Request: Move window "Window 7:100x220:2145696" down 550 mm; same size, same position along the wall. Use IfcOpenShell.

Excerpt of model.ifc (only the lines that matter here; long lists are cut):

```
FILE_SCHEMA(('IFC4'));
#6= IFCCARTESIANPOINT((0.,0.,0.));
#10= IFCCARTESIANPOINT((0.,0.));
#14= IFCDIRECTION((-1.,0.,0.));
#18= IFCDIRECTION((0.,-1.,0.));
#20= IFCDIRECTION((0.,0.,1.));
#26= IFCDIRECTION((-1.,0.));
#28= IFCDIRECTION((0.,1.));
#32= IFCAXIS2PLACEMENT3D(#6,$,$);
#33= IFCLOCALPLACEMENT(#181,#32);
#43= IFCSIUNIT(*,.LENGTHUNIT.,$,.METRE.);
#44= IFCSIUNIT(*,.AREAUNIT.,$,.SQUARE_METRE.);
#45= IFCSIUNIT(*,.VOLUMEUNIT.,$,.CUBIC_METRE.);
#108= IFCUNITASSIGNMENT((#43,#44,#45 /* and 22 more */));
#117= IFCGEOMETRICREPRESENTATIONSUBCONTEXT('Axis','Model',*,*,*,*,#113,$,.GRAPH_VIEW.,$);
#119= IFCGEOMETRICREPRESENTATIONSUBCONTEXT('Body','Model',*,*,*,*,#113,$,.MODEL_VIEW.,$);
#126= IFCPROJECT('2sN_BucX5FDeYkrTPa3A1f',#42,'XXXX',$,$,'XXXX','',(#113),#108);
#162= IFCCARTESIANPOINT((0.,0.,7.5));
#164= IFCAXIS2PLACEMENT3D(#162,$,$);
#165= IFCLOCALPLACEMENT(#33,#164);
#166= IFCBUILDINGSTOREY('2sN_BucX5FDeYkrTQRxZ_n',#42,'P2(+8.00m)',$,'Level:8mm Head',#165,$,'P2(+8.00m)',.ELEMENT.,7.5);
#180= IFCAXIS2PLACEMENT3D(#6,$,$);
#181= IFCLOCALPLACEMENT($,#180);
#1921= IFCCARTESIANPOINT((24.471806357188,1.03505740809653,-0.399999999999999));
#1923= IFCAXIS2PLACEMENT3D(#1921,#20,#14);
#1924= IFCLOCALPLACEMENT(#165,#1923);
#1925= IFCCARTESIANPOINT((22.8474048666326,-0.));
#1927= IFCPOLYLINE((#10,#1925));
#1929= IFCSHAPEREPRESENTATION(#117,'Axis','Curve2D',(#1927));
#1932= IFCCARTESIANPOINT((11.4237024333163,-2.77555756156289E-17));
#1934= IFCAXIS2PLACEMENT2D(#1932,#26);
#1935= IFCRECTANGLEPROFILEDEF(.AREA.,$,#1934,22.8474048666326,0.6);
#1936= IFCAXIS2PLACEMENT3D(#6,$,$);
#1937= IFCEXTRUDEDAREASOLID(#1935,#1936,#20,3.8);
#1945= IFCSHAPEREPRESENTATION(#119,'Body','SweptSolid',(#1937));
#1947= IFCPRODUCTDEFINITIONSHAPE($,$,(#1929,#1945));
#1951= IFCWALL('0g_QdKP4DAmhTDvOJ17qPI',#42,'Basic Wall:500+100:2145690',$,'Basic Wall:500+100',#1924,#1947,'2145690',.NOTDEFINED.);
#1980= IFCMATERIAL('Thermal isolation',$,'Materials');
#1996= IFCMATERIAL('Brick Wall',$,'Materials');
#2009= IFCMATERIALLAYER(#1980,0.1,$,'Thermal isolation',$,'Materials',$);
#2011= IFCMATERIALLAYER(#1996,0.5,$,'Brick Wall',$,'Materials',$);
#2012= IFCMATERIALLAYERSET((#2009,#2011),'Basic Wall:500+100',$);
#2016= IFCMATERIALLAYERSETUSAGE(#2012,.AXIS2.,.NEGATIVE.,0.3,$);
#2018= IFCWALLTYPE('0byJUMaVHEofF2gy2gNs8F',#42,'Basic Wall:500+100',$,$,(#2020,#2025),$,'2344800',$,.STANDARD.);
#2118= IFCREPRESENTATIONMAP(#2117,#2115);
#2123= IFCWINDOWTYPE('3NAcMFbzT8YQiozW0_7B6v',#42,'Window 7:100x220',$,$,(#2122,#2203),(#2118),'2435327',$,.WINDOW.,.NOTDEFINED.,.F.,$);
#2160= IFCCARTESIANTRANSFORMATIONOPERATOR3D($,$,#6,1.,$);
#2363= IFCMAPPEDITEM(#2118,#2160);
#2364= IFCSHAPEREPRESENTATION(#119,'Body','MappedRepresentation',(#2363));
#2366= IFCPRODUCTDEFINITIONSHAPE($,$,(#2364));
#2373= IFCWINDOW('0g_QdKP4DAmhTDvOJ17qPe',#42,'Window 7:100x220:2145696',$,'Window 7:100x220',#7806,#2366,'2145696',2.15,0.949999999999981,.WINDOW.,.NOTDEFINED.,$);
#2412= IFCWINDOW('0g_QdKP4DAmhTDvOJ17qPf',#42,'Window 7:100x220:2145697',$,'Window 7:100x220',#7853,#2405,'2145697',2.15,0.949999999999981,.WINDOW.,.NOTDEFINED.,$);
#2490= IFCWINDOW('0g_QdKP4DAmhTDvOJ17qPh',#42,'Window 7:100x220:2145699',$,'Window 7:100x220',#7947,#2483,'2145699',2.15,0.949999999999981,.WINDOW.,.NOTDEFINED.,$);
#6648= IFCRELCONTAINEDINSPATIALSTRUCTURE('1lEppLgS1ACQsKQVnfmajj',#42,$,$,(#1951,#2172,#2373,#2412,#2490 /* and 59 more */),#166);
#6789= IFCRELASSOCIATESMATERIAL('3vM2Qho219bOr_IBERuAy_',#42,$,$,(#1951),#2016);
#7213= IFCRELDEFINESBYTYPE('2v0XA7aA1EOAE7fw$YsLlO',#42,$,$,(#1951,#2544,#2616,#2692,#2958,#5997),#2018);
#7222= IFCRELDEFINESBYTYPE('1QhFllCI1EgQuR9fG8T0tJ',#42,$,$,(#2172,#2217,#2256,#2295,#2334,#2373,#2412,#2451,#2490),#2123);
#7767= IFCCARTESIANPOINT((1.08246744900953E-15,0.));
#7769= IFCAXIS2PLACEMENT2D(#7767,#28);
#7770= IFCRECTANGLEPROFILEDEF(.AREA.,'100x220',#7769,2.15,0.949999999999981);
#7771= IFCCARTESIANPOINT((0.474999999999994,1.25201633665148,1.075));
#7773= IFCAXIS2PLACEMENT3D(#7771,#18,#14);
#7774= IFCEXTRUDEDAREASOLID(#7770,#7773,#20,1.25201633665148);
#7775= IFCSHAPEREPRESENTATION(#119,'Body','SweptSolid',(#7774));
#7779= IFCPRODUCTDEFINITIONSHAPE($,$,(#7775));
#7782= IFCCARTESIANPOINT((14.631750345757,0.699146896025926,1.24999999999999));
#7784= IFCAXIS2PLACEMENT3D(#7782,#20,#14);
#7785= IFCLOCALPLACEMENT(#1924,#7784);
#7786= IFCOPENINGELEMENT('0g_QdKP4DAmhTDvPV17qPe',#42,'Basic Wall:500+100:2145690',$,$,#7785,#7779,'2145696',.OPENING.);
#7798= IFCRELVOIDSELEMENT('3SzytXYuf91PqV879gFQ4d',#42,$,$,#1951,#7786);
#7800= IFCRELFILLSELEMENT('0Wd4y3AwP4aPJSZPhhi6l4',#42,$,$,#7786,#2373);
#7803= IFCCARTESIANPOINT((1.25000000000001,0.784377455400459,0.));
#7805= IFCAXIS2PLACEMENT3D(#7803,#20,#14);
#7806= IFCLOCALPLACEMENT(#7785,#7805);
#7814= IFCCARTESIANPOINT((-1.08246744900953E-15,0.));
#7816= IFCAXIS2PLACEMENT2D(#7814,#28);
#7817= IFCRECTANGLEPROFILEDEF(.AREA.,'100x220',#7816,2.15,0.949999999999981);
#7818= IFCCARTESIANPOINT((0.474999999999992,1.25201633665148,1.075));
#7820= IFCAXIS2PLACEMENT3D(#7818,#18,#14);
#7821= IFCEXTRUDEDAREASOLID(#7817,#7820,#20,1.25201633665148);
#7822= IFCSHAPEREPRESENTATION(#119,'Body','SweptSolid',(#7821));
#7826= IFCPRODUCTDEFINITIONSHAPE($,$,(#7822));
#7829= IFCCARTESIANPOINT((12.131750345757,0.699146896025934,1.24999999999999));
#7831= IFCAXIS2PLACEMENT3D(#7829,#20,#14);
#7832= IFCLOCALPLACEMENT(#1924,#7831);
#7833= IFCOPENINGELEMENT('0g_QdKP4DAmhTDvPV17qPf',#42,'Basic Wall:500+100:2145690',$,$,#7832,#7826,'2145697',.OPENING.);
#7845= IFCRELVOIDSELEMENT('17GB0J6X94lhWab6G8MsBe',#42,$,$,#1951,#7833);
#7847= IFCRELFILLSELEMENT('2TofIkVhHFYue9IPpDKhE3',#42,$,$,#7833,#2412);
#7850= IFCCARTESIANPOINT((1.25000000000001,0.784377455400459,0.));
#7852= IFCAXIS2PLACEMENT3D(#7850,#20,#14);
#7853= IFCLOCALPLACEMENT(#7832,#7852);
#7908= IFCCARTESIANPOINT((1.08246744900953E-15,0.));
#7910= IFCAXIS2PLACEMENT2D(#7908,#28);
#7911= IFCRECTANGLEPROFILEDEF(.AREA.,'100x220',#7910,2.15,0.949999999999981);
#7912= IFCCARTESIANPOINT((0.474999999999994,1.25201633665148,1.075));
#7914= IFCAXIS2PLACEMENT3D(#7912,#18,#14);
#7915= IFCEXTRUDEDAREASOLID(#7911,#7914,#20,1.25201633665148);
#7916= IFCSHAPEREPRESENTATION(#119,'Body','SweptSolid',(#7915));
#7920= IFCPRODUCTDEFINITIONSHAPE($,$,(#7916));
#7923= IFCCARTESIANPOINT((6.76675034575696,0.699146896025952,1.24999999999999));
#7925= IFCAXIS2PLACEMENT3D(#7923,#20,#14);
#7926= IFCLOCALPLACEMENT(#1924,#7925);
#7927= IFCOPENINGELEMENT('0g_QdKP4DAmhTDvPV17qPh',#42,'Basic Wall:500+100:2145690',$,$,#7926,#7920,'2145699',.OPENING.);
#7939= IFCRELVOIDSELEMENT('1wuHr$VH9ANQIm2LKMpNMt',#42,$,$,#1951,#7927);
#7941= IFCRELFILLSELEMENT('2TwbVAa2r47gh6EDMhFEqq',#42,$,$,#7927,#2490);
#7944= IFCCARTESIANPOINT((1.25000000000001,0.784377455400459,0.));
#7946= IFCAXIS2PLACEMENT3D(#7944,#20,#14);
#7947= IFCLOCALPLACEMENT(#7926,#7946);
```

```python
import numpy as np
import ifcopenshell
import ifcopenshell.api.geometry
import ifcopenshell.util.placement
import ifcopenshell.util.unit

model = ifcopenshell.open("model.ifc")
unit_scale = ifcopenshell.util.unit.calculate_unit_scale(model)

window = model.by_id(2373)
opening = window.FillsVoids[0].RelatingOpeningElement
dz = -0.55

shift = np.array([0.0, 0.0, dz])
# The window is placed relative to its opening, so it follows when the opening moves.
matrix = ifcopenshell.util.placement.get_local_placement(opening.ObjectPlacement)
matrix[:3, 3] += shift
ifcopenshell.api.geometry.edit_object_placement(
    model, product=opening, matrix=matrix, is_si=False, should_transform_children=True
)

print(f"moved by {dz * unit_scale:+.3f} m")

model.write("model_rev.ifc")
```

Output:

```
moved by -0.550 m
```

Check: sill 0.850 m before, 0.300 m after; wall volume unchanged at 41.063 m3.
